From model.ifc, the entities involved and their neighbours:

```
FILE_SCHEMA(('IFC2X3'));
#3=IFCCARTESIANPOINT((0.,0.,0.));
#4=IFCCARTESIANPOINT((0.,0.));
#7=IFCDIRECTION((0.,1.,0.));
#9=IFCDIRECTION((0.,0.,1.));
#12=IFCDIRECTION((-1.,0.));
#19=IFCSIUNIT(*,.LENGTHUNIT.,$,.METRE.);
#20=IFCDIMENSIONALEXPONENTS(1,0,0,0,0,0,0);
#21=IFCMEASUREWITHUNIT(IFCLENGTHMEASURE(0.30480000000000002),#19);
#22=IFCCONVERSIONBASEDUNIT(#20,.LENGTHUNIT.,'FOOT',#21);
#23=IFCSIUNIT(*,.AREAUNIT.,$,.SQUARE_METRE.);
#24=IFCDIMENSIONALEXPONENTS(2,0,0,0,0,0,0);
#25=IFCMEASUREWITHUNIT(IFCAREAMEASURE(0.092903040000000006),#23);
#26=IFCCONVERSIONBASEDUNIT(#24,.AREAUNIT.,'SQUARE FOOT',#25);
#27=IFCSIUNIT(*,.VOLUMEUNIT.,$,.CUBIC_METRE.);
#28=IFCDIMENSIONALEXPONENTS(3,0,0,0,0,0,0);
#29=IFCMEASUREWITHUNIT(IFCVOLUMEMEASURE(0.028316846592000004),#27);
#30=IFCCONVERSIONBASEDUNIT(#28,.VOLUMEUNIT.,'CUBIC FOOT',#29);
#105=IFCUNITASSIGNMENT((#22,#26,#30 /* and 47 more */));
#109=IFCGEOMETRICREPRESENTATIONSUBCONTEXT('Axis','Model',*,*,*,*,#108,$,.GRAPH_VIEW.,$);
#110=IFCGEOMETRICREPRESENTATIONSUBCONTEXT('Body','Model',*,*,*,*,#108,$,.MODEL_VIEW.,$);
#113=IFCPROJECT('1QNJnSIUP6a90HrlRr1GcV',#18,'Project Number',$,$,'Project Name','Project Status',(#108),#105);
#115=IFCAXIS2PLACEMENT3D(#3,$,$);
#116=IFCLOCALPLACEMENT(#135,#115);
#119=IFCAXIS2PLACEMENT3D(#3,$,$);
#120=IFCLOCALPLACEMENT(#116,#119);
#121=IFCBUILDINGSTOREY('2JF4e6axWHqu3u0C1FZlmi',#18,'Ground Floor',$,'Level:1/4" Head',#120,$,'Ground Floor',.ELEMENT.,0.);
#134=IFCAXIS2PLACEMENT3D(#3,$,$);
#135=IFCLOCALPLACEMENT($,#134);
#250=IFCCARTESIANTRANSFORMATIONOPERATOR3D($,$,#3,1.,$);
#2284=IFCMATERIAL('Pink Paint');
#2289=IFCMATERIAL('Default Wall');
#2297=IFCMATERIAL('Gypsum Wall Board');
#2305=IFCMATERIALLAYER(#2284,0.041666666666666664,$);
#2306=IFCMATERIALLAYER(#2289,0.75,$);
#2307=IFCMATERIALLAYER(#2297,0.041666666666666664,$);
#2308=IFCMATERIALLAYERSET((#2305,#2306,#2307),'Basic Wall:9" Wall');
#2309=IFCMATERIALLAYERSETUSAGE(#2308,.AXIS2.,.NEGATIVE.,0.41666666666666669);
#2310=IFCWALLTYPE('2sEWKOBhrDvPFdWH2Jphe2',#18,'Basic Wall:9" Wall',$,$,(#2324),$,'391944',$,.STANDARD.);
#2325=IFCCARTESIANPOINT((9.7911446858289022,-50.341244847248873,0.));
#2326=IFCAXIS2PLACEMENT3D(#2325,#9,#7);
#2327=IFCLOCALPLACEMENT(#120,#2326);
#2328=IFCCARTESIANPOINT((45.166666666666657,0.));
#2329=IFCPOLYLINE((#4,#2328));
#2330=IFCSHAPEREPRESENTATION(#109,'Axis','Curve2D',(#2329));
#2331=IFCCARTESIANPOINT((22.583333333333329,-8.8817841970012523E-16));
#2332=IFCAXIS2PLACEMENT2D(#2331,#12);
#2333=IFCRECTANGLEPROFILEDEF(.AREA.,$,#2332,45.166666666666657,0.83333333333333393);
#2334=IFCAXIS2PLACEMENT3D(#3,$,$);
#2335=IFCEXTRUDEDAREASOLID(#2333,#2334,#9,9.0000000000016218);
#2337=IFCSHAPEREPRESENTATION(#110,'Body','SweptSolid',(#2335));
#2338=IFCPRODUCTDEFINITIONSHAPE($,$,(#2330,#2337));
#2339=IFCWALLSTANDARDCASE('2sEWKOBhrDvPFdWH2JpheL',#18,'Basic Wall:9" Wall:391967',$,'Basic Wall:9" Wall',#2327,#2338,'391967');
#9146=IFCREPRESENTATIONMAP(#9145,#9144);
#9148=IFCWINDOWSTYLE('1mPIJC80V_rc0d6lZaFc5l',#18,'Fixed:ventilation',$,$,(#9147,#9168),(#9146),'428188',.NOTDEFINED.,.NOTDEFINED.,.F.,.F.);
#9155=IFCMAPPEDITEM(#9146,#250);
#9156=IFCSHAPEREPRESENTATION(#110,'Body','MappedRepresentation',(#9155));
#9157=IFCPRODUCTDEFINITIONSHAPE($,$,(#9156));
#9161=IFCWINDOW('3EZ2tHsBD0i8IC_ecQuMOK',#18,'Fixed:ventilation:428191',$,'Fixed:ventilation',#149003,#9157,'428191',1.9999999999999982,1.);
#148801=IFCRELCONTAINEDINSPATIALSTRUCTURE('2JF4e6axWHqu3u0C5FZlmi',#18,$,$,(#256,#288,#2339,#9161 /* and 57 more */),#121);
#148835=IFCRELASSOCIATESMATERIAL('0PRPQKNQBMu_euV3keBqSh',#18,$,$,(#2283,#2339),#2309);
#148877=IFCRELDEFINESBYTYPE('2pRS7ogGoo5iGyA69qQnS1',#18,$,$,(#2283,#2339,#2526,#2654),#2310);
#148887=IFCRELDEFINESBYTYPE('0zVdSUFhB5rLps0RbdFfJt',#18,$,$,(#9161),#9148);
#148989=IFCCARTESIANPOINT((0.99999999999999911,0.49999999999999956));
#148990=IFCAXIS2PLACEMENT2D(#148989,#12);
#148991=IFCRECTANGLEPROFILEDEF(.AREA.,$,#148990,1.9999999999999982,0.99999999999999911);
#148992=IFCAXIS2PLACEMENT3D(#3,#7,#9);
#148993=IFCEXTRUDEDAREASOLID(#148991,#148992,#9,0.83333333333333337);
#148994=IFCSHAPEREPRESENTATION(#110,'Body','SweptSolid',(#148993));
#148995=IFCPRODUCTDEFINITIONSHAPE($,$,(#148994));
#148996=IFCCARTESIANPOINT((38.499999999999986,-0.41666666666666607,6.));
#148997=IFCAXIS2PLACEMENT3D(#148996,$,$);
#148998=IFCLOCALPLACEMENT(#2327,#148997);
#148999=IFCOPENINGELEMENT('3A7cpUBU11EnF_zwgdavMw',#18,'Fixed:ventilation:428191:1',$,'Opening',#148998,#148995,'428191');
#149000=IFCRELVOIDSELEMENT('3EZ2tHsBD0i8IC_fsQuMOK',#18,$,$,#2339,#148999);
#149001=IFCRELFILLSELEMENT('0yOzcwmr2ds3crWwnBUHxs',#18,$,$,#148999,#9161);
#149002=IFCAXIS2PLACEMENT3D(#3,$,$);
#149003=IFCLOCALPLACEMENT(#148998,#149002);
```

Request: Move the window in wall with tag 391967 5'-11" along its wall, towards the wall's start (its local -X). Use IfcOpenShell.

```python
import ifcopenshell
import ifcopenshell.api.geometry
import ifcopenshell.util.placement
import ifcopenshell.util.unit

model = ifcopenshell.open("model.ifc")
unit_scale = ifcopenshell.util.unit.calculate_unit_scale(model)

window = model.by_guid("3EZ2tHsBD0i8IC_ecQuMOK")
opening = window.FillsVoids[0].RelatingOpeningElement
wall = opening.VoidsElements[0].RelatingBuildingElement

wall_matrix = ifcopenshell.util.placement.get_local_placement(wall.ObjectPlacement)
shift = wall_matrix[:3, 0] * -71 * 0.0254 / unit_scale
before = ifcopenshell.util.placement.get_local_placement(window.ObjectPlacement)[:3, 3].copy()

# The window is placed relative to its opening, so it follows when the opening moves.
matrix = ifcopenshell.util.placement.get_local_placement(opening.ObjectPlacement)
matrix[:3, 3] += shift
ifcopenshell.api.geometry.edit_object_placement(
    model, product=opening, matrix=matrix, is_si=False, should_transform_children=True
)

after = ifcopenshell.util.placement.get_local_placement(window.ObjectPlacement)[:3, 3]
print("window moved by", (after - before).round(3) + 0.0)

model.write("model_edited.ifc")
```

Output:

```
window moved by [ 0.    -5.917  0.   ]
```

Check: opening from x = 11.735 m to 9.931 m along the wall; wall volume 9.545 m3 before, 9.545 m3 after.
